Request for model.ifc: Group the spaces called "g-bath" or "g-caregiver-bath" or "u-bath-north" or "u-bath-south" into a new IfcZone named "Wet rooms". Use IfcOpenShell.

First a look at what the model holds.

```python
import ifcopenshell

model = ifcopenshell.open("model.ifc")
print(model.schema)
seen = {}
for space in model.by_type("IfcSpace"):
    seen[space.LongName] = seen.get(space.LongName, 0) + 1
for name, count in sorted(seen.items(), key=str):
    print(count, "x", name)
print("zones:", [z.Name for z in model.by_type("IfcZone")][:20])
```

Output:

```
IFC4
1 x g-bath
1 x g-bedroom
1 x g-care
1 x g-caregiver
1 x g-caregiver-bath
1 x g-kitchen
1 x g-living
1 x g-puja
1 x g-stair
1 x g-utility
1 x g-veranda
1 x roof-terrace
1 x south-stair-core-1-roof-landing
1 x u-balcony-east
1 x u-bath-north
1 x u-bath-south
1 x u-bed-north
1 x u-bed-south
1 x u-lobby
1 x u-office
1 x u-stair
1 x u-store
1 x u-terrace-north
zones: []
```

```python
import ifcopenshell
import ifcopenshell.api.group
import ifcopenshell.api.root

model = ifcopenshell.open("model.ifc")

names = {"g-bath", "g-caregiver-bath", "u-bath-north", "u-bath-south"}
spaces = [s for s in model.by_type("IfcSpace") if s.LongName in names]

zone = ifcopenshell.api.root.create_entity(model, ifc_class="IfcZone", name="Wet rooms")
ifcopenshell.api.group.assign_group(model, products=spaces, group=zone)
print(len(spaces), "spaces in", zone.Name)

model.write("model_updated.ifc")
```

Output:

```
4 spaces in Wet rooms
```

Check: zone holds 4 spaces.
